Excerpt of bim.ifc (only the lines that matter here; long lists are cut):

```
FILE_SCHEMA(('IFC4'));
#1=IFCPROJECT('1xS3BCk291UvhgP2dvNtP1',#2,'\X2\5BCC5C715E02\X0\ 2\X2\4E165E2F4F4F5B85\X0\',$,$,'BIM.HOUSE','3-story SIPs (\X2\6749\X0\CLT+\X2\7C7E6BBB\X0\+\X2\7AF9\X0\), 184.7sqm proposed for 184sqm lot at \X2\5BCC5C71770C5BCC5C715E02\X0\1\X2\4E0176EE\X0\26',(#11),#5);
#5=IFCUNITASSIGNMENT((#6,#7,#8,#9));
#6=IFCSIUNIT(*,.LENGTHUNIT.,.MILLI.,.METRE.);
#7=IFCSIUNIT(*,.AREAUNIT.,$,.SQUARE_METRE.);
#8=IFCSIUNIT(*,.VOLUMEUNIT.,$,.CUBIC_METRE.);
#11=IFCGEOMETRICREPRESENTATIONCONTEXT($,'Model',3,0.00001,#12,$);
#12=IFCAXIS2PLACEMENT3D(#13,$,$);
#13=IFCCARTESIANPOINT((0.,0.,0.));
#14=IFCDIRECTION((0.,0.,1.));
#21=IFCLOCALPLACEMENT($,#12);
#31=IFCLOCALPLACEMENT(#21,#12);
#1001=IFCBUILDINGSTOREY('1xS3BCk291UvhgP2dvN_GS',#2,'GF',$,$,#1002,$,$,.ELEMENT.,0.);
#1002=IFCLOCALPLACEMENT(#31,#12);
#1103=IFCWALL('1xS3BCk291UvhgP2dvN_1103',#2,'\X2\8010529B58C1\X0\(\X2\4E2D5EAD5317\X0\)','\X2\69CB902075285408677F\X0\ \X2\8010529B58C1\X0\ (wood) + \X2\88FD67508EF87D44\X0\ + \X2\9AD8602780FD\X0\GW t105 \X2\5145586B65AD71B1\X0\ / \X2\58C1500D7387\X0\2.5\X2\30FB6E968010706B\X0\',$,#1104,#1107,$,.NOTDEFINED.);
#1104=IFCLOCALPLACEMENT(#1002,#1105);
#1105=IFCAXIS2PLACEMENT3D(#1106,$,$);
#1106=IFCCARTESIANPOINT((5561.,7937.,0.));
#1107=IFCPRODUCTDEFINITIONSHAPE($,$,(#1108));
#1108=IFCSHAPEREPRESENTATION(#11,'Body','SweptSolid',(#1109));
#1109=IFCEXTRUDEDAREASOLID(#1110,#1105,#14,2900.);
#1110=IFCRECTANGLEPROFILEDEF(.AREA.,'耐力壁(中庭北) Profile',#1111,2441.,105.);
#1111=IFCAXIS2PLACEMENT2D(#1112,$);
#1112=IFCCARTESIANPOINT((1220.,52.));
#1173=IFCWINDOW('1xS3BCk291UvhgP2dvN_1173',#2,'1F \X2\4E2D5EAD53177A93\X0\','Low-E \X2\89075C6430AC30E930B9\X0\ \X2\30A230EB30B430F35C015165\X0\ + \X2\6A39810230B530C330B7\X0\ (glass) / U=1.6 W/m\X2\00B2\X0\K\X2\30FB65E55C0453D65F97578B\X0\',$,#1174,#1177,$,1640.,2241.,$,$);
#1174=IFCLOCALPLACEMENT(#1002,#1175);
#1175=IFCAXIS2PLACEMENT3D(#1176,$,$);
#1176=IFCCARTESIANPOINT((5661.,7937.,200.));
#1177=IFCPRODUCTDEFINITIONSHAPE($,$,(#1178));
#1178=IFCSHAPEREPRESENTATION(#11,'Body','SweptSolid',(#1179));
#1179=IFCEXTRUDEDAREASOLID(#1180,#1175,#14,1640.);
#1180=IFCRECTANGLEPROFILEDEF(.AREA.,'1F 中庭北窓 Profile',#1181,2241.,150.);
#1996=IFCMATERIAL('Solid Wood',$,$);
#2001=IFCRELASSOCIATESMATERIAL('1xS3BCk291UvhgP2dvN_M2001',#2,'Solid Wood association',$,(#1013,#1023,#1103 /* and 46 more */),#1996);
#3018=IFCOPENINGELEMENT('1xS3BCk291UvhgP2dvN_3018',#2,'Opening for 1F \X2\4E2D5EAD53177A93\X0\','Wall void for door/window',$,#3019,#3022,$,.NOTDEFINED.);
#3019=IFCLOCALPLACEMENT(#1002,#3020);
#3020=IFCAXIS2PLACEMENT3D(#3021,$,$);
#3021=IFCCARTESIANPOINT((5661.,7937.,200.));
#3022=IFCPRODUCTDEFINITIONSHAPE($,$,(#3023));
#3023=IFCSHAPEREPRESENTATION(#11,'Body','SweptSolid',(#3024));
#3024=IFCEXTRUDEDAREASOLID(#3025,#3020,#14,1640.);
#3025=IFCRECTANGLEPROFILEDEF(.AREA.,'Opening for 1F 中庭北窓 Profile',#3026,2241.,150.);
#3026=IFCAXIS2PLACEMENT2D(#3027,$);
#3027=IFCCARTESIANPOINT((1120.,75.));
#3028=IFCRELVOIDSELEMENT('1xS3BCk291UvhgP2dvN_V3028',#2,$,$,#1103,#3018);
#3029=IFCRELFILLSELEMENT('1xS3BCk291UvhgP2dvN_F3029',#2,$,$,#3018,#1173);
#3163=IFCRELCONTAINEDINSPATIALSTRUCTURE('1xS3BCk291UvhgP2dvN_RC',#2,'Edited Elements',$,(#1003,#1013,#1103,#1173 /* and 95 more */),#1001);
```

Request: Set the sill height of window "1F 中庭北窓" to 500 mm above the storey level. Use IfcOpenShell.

```python
import numpy as np
import ifcopenshell
import ifcopenshell.api.geometry
import ifcopenshell.geom
import ifcopenshell.util.element
import ifcopenshell.util.placement
import ifcopenshell.util.shape
import ifcopenshell.util.unit

model = ifcopenshell.open("bim.ifc")
unit_scale = ifcopenshell.util.unit.calculate_unit_scale(model)

window = model.by_guid("1xS3BCk291UvhgP2dvN_1173")
opening = window.FillsVoids[0].RelatingOpeningElement
storey = ifcopenshell.util.element.get_container(window, ifc_class="IfcBuildingStorey")
level = ifcopenshell.util.placement.get_local_placement(storey.ObjectPlacement)[2, 3]

# The opening's origin need not be at the sill, so measure its lowest point.
shape = ifcopenshell.geom.create_shape(ifcopenshell.geom.settings(), opening)
bottom = ifcopenshell.util.shape.get_shape_bottom_elevation(shape, shape.geometry) / unit_scale
dz = level + 500.0 - bottom

shift = np.array([0.0, 0.0, dz])
# The window is not placed relative to its opening, so move both.
for product in (opening, window):
    matrix = ifcopenshell.util.placement.get_local_placement(product.ObjectPlacement)
    matrix[:3, 3] += shift
    ifcopenshell.api.geometry.edit_object_placement(model, product=product, matrix=matrix, is_si=False)

print(f"moved by {dz * unit_scale:+.3f} m")

model.write("bim_updated.ifc")
```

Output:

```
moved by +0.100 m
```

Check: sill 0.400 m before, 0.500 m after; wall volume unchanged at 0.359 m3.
